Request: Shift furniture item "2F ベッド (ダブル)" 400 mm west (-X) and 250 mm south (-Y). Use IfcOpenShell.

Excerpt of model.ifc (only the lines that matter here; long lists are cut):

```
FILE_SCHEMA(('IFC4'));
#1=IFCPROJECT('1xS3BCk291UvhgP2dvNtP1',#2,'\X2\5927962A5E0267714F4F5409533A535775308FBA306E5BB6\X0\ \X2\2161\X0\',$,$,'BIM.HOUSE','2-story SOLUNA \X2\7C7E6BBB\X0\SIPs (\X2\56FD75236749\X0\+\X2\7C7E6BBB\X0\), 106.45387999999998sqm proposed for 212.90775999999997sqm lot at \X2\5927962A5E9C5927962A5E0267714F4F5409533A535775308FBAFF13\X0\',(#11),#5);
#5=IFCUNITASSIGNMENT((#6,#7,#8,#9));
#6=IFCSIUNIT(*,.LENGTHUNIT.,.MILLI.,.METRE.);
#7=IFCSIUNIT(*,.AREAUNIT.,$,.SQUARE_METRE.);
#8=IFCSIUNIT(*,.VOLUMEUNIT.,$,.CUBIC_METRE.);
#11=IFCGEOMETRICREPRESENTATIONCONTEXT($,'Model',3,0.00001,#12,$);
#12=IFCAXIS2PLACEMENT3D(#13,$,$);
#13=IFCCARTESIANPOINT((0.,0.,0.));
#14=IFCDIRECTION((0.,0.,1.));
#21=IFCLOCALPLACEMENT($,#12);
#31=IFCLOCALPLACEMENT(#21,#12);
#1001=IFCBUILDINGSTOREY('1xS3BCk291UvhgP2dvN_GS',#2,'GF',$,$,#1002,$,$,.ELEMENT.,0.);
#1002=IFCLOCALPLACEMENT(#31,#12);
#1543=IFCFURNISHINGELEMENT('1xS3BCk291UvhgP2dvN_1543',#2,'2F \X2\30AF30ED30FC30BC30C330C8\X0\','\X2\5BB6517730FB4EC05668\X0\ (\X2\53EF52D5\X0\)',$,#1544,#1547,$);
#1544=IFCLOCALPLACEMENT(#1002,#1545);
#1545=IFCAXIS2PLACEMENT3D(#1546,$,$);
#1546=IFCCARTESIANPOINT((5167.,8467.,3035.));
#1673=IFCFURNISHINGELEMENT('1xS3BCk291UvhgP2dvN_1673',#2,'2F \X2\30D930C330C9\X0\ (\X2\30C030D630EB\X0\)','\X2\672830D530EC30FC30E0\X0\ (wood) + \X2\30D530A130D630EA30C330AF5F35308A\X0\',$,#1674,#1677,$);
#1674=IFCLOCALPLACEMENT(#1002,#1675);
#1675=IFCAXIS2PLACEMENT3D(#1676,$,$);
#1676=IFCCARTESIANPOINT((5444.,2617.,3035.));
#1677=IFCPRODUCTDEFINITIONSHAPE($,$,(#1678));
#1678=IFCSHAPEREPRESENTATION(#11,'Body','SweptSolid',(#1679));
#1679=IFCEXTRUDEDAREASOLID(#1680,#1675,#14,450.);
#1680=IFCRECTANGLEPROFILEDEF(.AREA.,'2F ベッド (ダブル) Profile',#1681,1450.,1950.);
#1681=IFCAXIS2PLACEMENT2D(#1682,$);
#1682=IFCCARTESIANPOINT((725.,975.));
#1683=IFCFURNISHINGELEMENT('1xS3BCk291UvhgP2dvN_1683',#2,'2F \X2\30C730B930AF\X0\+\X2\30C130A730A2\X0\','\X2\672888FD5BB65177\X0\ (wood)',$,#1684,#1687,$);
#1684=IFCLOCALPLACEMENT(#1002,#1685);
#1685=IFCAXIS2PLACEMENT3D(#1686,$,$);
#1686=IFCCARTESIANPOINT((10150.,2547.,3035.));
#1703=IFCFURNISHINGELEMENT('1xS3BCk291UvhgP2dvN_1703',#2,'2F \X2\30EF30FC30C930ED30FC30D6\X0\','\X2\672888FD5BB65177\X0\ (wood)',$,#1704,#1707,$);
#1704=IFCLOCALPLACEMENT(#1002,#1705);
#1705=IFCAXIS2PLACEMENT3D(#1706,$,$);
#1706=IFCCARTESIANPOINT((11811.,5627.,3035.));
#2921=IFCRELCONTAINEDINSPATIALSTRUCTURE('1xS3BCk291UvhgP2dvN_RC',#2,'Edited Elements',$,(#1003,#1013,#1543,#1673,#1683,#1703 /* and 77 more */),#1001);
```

```python
import ifcopenshell
import ifcopenshell.api.geometry
import ifcopenshell.util.placement
import ifcopenshell.util.unit

model = ifcopenshell.open("model.ifc")
unit_scale = ifcopenshell.util.unit.calculate_unit_scale(model)

item = model.by_id(1673)
matrix = ifcopenshell.util.placement.get_local_placement(item.ObjectPlacement)
matrix[0, 3] -= 0.4 / unit_scale
matrix[1, 3] -= 0.25 / unit_scale
ifcopenshell.api.geometry.edit_object_placement(model, product=item, matrix=matrix, is_si=False)

print(ifcopenshell.util.placement.get_local_placement(item.ObjectPlacement).round(3) + 0.0)

model.write("model_edited.ifc")
```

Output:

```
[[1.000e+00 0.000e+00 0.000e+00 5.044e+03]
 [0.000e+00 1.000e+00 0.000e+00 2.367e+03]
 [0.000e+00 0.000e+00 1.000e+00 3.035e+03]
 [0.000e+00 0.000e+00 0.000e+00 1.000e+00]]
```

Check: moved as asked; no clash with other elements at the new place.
